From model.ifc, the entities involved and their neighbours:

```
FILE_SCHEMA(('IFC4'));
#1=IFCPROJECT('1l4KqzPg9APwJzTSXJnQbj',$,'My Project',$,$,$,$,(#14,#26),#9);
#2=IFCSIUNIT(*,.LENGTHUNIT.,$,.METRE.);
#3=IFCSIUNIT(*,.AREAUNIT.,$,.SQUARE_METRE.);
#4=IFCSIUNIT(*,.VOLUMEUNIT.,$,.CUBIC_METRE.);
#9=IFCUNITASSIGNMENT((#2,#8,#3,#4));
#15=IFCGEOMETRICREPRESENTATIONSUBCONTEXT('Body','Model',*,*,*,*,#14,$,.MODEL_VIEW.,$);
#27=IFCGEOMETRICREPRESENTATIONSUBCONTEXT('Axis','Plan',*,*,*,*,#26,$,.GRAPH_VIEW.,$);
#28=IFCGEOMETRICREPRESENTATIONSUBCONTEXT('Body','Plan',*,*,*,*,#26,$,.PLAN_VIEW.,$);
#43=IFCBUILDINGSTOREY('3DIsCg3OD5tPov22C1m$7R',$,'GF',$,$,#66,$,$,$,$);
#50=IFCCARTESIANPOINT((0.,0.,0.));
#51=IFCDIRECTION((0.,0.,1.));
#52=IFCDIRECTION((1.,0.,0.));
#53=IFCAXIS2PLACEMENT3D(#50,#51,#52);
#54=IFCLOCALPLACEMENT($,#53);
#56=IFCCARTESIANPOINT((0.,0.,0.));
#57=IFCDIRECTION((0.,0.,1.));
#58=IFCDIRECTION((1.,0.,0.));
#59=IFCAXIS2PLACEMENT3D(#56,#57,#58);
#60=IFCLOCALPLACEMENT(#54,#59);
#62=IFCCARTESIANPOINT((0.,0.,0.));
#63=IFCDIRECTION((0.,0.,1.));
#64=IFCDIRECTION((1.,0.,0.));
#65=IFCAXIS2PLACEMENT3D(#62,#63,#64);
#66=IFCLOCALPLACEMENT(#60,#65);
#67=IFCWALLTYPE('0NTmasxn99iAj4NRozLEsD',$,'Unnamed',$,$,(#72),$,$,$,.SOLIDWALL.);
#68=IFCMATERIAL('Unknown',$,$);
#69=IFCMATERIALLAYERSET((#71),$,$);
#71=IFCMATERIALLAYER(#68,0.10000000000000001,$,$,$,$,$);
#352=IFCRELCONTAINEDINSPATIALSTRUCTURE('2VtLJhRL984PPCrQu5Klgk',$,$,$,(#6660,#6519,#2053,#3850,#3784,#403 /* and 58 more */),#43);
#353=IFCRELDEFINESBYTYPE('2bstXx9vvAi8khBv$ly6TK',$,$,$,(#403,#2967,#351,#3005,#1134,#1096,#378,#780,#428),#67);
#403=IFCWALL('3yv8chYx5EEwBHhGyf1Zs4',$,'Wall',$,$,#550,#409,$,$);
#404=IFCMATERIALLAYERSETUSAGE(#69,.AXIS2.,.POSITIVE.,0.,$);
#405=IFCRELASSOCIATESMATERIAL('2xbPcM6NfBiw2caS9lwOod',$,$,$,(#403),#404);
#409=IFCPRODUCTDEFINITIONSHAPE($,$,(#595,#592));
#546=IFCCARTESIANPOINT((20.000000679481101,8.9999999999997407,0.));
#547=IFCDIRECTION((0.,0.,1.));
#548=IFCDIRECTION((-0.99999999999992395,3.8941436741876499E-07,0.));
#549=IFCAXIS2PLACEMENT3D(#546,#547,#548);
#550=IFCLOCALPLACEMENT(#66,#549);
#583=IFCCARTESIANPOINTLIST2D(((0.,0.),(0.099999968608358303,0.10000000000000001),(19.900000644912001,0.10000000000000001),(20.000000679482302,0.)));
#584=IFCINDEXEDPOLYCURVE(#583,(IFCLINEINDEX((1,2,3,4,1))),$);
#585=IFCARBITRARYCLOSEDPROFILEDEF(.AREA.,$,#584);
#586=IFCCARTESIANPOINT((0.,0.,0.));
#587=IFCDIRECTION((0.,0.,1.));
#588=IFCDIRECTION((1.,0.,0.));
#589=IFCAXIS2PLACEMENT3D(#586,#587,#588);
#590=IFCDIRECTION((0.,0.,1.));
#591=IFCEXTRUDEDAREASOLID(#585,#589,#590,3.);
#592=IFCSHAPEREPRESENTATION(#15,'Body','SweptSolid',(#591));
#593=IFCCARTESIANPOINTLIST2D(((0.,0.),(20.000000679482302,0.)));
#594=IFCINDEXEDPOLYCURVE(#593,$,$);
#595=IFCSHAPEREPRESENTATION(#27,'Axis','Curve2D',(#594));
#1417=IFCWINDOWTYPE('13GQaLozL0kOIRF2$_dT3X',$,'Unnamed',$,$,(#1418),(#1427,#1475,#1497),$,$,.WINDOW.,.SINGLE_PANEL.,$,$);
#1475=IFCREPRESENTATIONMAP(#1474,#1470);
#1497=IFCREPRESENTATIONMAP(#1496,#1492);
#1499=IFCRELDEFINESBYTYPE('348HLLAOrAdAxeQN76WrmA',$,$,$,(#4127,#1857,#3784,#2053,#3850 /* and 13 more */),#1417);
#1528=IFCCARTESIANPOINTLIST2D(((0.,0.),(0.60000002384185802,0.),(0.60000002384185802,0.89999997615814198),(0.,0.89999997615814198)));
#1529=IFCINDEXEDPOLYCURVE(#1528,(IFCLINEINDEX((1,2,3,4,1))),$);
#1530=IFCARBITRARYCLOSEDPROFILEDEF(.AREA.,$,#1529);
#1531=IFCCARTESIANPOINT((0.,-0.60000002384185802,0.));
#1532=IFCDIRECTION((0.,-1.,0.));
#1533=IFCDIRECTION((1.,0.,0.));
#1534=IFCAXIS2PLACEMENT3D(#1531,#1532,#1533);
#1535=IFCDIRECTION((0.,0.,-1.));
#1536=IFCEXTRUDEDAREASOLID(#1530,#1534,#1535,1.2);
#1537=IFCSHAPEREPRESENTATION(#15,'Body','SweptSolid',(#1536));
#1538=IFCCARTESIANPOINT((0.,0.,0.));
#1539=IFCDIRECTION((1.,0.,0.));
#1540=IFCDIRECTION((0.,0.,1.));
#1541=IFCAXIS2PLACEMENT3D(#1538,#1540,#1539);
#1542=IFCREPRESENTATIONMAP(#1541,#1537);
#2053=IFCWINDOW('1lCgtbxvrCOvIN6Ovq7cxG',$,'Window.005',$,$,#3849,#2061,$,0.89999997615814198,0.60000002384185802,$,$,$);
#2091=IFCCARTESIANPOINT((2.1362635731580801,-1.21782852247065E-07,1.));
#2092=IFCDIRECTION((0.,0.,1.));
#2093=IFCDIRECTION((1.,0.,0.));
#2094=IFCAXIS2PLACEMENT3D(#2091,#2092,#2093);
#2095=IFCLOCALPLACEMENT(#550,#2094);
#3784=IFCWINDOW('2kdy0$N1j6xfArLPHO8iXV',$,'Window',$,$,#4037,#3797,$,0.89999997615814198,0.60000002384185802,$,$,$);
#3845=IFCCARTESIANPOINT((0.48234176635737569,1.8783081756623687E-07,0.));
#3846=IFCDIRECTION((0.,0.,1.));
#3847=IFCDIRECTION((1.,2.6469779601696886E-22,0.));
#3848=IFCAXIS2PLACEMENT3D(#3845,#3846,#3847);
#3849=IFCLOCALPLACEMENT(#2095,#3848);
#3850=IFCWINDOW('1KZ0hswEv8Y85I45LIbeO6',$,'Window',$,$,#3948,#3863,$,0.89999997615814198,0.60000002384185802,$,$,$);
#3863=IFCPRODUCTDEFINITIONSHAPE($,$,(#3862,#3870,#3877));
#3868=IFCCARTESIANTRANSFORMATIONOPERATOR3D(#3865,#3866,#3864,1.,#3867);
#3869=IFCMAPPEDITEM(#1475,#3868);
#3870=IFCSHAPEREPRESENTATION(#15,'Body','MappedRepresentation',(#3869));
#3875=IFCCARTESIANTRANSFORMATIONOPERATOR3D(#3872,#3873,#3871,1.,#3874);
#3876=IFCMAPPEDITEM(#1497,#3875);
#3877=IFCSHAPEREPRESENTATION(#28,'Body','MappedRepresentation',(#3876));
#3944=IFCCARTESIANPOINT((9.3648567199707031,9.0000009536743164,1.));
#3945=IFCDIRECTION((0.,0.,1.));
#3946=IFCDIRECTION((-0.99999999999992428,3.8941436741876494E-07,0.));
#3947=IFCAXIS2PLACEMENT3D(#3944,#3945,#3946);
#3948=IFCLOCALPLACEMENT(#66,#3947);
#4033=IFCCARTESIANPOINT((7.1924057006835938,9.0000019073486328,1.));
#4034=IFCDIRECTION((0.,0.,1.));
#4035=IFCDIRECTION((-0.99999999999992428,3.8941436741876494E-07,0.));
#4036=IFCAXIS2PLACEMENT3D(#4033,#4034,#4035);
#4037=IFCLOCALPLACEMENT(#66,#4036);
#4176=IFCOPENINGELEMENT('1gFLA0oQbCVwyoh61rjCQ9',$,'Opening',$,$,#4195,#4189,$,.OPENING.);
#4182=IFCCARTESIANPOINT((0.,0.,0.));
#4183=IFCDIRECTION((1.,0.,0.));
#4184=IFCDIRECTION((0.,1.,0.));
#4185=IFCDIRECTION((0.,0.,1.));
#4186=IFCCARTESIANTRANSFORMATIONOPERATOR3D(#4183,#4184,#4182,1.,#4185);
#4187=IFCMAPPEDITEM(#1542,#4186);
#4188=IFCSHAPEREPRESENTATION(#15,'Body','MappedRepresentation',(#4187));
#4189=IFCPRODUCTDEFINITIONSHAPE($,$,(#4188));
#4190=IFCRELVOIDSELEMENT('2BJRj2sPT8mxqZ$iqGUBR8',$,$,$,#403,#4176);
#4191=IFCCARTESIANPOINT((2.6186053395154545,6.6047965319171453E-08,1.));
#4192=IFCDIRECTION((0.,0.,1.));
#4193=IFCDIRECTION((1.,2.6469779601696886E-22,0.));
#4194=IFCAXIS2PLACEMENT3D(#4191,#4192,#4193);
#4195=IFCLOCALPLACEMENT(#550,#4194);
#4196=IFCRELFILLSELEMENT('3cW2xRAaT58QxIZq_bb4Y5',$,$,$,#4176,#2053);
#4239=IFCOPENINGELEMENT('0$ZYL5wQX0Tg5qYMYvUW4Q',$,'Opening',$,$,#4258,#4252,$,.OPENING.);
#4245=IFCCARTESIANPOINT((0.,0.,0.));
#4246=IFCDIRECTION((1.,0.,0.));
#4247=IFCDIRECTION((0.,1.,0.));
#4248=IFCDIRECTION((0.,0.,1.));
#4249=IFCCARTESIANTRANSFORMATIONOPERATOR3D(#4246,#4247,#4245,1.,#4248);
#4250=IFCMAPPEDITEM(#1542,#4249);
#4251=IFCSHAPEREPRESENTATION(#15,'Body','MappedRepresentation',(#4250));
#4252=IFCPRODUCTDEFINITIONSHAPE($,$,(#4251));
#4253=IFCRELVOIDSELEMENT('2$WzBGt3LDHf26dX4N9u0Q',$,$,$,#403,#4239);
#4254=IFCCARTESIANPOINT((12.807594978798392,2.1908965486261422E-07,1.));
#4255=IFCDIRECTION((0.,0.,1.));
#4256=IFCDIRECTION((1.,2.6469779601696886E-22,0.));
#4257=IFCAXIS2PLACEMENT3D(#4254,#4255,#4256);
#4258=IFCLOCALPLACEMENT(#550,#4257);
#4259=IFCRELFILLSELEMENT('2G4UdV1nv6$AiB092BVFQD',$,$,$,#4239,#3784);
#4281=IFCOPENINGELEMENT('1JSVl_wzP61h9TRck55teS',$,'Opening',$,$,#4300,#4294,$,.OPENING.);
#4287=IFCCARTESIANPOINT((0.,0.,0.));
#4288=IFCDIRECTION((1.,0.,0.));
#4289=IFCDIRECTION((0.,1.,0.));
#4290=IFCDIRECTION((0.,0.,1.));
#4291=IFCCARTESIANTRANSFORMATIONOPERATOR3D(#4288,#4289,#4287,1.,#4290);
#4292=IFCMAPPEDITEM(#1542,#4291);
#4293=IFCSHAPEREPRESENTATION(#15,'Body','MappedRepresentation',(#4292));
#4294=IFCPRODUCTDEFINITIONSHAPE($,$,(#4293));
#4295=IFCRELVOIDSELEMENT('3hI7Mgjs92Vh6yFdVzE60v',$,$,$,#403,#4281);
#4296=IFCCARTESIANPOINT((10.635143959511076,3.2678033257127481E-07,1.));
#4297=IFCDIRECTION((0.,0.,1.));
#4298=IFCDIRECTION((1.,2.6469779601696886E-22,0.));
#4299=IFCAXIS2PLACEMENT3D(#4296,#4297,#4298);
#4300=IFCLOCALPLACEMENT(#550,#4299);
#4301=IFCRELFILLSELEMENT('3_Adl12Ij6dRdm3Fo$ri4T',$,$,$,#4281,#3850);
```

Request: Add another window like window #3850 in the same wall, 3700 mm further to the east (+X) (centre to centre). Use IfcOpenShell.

```python
import ifcopenshell
import ifcopenshell.api.feature
import ifcopenshell.api.geometry
import ifcopenshell.api.root
import ifcopenshell.geom
import ifcopenshell.util.element
import ifcopenshell.util.placement
import ifcopenshell.util.shape

model = ifcopenshell.open("model.ifc")
settings = ifcopenshell.geom.settings()


def volume(element):
    """Net volume in cubic metres, openings subtracted."""
    shape = ifcopenshell.geom.create_shape(settings, element)
    return ifcopenshell.util.shape.get_volume(shape.geometry)


window = model.by_guid("1KZ0hswEv8Y85I45LIbeO6")
opening = window.FillsVoids[0].RelatingOpeningElement
wall = opening.VoidsElements[0].RelatingBuildingElement
before = volume(wall)
shift = ifcopenshell.util.placement.get_local_placement(wall.ObjectPlacement)[:3, 0] * -3.7

# copy_class copies the void relationship, type, container and properties, but no geometry.
new_opening = ifcopenshell.api.root.copy_class(model, product=opening)
new_opening.Representation = ifcopenshell.util.element.copy_deep(
    model, opening.Representation, exclude=["IfcGeometricRepresentationContext", "IfcRepresentationMap"]
)
new_window = ifcopenshell.api.root.copy_class(model, product=window)
new_window.Representation = ifcopenshell.util.element.copy_deep(
    model, window.Representation, exclude=["IfcGeometricRepresentationContext", "IfcRepresentationMap"]
)
ifcopenshell.api.feature.add_filling(model, opening=new_opening, element=new_window)

for old, new in ((opening, new_opening), (window, new_window)):
    matrix = ifcopenshell.util.placement.get_local_placement(old.ObjectPlacement)
    matrix[:3, 3] += shift
    ifcopenshell.api.geometry.edit_object_placement(model, product=new, matrix=matrix, is_si=False)

after = volume(wall)

print(f"wall volume {before:.3f} -> {after:.3f} m3")

model.write("model_rev.ifc")
```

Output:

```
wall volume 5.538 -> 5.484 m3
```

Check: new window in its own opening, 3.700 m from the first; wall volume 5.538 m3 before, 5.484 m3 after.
